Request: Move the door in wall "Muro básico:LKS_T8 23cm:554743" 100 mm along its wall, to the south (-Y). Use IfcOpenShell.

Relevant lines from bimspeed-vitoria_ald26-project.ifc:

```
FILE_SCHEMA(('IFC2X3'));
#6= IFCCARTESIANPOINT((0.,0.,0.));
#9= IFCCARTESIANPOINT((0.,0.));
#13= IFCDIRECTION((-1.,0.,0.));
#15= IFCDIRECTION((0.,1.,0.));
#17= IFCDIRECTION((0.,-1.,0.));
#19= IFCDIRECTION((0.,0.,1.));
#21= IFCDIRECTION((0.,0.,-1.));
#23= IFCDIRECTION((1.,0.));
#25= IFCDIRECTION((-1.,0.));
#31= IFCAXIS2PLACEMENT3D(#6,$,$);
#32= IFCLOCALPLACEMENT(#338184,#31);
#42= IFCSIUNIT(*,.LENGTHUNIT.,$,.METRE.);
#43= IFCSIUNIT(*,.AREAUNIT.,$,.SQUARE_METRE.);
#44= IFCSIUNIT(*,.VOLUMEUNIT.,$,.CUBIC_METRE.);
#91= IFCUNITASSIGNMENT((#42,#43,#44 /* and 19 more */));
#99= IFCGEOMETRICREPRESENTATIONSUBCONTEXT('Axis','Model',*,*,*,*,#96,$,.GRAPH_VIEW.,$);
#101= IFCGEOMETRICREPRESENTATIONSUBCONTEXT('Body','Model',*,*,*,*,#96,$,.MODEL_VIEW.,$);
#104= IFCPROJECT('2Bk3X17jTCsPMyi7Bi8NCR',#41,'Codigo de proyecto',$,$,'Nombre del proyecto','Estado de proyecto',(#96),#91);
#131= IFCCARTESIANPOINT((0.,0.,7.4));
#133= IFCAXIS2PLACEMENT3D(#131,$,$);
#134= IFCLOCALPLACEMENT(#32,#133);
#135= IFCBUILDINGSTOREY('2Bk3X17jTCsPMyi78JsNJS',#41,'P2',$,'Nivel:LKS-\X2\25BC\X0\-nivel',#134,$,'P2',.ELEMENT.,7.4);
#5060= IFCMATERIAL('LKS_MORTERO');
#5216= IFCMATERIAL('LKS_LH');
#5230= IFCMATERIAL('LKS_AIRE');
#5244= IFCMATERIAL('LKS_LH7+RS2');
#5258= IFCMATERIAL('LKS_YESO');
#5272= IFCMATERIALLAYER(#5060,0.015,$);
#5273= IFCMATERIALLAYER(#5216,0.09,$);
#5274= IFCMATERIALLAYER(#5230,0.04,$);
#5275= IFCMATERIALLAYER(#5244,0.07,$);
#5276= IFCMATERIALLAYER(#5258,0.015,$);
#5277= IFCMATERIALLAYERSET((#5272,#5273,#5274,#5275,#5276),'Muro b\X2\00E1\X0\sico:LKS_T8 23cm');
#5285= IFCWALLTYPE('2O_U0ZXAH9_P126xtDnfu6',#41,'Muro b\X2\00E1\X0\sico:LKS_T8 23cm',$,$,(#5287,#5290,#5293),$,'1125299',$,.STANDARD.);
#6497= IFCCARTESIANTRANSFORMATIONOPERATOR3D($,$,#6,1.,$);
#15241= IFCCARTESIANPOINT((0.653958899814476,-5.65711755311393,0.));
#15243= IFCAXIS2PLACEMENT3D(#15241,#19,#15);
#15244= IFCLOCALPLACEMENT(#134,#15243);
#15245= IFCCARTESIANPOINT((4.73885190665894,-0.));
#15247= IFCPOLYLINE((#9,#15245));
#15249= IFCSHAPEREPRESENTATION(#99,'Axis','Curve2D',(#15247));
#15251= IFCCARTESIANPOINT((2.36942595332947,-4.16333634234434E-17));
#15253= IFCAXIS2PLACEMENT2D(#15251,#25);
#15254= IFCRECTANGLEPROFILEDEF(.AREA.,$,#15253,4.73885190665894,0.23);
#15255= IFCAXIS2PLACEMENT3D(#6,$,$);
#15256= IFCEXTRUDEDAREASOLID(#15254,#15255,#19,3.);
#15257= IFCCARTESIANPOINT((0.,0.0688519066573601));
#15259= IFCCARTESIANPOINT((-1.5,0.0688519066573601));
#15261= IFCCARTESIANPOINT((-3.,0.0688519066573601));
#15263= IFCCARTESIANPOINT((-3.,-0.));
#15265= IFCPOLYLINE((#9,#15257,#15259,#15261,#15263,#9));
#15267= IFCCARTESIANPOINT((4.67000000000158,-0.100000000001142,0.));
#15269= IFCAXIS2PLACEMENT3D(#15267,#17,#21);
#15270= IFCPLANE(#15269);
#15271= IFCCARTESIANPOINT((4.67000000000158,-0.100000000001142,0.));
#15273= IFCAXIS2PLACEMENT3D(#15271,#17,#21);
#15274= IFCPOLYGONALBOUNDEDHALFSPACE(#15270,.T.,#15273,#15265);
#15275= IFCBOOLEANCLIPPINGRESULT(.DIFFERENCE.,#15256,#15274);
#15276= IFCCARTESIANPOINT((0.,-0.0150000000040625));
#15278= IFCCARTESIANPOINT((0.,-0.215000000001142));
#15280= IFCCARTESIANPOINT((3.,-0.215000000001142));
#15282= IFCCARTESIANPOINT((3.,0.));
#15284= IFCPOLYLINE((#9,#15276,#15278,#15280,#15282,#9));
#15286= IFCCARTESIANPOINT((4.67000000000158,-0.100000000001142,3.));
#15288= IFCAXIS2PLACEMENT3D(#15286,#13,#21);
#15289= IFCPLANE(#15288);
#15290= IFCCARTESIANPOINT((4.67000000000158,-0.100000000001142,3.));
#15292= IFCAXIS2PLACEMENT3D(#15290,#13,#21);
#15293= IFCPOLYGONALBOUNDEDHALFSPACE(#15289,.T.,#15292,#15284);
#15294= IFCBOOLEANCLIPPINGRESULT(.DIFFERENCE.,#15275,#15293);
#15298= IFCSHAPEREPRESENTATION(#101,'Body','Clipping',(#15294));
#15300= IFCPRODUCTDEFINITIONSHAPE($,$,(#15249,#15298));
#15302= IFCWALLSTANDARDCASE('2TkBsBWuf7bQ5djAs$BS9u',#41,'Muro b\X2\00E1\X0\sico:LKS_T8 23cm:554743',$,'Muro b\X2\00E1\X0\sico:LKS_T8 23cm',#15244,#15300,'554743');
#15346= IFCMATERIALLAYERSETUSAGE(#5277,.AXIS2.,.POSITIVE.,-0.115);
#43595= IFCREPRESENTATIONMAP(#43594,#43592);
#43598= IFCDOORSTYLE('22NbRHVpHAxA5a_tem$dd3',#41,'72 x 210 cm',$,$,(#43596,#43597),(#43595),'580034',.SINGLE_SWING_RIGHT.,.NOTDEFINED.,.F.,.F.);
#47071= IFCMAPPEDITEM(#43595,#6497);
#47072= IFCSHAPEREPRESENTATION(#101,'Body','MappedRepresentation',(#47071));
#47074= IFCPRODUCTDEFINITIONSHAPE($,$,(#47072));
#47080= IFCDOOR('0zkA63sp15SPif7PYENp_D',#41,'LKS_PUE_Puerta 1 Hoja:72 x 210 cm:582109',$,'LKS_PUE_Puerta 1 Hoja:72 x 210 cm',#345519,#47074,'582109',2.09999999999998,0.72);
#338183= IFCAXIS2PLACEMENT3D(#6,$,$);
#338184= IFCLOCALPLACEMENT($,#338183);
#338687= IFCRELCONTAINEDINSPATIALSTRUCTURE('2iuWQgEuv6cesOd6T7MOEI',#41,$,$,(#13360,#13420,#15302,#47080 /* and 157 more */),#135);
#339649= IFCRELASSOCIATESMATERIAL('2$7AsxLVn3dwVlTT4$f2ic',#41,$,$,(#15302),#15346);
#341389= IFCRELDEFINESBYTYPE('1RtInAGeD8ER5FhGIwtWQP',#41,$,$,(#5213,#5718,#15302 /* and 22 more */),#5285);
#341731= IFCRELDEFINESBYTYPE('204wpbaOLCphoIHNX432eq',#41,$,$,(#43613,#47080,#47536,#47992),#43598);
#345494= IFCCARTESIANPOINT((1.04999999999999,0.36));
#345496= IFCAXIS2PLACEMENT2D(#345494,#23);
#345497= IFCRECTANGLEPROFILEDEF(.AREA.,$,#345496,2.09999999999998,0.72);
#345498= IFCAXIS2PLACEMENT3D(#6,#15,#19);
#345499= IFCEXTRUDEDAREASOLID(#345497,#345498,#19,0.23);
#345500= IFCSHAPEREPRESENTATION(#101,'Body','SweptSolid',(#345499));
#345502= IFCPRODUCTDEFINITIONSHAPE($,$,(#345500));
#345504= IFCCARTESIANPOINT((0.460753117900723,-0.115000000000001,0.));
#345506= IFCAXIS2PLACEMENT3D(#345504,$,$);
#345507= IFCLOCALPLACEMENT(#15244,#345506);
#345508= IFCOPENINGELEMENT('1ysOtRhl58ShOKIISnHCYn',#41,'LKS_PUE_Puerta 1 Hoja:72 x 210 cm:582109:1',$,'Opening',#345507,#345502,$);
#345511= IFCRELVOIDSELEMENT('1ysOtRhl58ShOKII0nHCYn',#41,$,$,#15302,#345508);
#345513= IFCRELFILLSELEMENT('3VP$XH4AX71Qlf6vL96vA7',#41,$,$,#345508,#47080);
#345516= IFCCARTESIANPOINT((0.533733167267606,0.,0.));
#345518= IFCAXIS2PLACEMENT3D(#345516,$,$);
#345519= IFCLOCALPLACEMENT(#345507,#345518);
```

```python
import ifcopenshell
import ifcopenshell.api.geometry
import ifcopenshell.util.placement

model = ifcopenshell.open("bimspeed-vitoria_ald26-project.ifc")

door = model.by_guid("0zkA63sp15SPif7PYENp_D")
opening = door.FillsVoids[0].RelatingOpeningElement
wall = opening.VoidsElements[0].RelatingBuildingElement

wall_matrix = ifcopenshell.util.placement.get_local_placement(wall.ObjectPlacement)
shift = wall_matrix[:3, 0] * -0.1
before = ifcopenshell.util.placement.get_local_placement(door.ObjectPlacement)[:3, 3].copy()

# The door is placed relative to its opening, so it follows when the opening moves.
matrix = ifcopenshell.util.placement.get_local_placement(opening.ObjectPlacement)
matrix[:3, 3] += shift
ifcopenshell.api.geometry.edit_object_placement(
    model, product=opening, matrix=matrix, is_si=False, should_transform_children=True
)

after = ifcopenshell.util.placement.get_local_placement(door.ObjectPlacement)[:3, 3]
print("door moved by", (after - before).round(3) + 0.0)

model.write("bimspeed-vitoria_ald26-project_v2.ifc")
```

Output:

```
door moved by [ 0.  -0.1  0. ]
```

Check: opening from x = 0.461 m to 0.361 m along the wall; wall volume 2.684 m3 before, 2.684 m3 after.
